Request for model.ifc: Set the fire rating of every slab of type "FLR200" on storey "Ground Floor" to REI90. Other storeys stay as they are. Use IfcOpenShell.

First a look at what the model holds.

```python
import ifcopenshell
import ifcopenshell.util.element

model = ifcopenshell.open("model.ifc")
print(model.schema)
storey = next(s for s in model.by_type("IfcBuildingStorey") if s.Name == "Ground Floor")
slabs = [e for e in ifcopenshell.util.element.get_decomposition(storey) if e.is_a("IfcSlab")]
seen = {}
for e in slabs:
    element_type = ifcopenshell.util.element.get_type(e)
    key = (element_type.Name if element_type != e and element_type else None, ifcopenshell.util.element.get_pset(e, "Pset_SlabCommon", "FireRating"))
    seen[key] = seen.get(key, 0) + 1
for (name, value), count in sorted(seen.items(), key=str):
    print(count, "x", name, "|", value)
```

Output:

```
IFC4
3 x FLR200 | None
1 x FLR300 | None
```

```python
import ifcopenshell
import ifcopenshell.api.pset
import ifcopenshell.util.element

model = ifcopenshell.open("model.ifc")

storey = next(s for s in model.by_type("IfcBuildingStorey") if s.Name == "Ground Floor")
slabs = [e for e in ifcopenshell.util.element.get_decomposition(storey) if e.is_a("IfcSlab")]

count = 0
for e in slabs:
    element_type = ifcopenshell.util.element.get_type(e)
    if element_type in (None, e) or element_type.Name != "FLR200":
        continue
    # add_pset returns the element's existing set when there is one.
    pset = ifcopenshell.api.pset.add_pset(model, product=e, name="Pset_SlabCommon")
    ifcopenshell.api.pset.edit_pset(model, pset=pset, properties={"FireRating": "REI90"})
    count += 1

print(count, "slabs updated")

model.write("model_rev.ifc")
```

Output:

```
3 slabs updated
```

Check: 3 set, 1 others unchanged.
